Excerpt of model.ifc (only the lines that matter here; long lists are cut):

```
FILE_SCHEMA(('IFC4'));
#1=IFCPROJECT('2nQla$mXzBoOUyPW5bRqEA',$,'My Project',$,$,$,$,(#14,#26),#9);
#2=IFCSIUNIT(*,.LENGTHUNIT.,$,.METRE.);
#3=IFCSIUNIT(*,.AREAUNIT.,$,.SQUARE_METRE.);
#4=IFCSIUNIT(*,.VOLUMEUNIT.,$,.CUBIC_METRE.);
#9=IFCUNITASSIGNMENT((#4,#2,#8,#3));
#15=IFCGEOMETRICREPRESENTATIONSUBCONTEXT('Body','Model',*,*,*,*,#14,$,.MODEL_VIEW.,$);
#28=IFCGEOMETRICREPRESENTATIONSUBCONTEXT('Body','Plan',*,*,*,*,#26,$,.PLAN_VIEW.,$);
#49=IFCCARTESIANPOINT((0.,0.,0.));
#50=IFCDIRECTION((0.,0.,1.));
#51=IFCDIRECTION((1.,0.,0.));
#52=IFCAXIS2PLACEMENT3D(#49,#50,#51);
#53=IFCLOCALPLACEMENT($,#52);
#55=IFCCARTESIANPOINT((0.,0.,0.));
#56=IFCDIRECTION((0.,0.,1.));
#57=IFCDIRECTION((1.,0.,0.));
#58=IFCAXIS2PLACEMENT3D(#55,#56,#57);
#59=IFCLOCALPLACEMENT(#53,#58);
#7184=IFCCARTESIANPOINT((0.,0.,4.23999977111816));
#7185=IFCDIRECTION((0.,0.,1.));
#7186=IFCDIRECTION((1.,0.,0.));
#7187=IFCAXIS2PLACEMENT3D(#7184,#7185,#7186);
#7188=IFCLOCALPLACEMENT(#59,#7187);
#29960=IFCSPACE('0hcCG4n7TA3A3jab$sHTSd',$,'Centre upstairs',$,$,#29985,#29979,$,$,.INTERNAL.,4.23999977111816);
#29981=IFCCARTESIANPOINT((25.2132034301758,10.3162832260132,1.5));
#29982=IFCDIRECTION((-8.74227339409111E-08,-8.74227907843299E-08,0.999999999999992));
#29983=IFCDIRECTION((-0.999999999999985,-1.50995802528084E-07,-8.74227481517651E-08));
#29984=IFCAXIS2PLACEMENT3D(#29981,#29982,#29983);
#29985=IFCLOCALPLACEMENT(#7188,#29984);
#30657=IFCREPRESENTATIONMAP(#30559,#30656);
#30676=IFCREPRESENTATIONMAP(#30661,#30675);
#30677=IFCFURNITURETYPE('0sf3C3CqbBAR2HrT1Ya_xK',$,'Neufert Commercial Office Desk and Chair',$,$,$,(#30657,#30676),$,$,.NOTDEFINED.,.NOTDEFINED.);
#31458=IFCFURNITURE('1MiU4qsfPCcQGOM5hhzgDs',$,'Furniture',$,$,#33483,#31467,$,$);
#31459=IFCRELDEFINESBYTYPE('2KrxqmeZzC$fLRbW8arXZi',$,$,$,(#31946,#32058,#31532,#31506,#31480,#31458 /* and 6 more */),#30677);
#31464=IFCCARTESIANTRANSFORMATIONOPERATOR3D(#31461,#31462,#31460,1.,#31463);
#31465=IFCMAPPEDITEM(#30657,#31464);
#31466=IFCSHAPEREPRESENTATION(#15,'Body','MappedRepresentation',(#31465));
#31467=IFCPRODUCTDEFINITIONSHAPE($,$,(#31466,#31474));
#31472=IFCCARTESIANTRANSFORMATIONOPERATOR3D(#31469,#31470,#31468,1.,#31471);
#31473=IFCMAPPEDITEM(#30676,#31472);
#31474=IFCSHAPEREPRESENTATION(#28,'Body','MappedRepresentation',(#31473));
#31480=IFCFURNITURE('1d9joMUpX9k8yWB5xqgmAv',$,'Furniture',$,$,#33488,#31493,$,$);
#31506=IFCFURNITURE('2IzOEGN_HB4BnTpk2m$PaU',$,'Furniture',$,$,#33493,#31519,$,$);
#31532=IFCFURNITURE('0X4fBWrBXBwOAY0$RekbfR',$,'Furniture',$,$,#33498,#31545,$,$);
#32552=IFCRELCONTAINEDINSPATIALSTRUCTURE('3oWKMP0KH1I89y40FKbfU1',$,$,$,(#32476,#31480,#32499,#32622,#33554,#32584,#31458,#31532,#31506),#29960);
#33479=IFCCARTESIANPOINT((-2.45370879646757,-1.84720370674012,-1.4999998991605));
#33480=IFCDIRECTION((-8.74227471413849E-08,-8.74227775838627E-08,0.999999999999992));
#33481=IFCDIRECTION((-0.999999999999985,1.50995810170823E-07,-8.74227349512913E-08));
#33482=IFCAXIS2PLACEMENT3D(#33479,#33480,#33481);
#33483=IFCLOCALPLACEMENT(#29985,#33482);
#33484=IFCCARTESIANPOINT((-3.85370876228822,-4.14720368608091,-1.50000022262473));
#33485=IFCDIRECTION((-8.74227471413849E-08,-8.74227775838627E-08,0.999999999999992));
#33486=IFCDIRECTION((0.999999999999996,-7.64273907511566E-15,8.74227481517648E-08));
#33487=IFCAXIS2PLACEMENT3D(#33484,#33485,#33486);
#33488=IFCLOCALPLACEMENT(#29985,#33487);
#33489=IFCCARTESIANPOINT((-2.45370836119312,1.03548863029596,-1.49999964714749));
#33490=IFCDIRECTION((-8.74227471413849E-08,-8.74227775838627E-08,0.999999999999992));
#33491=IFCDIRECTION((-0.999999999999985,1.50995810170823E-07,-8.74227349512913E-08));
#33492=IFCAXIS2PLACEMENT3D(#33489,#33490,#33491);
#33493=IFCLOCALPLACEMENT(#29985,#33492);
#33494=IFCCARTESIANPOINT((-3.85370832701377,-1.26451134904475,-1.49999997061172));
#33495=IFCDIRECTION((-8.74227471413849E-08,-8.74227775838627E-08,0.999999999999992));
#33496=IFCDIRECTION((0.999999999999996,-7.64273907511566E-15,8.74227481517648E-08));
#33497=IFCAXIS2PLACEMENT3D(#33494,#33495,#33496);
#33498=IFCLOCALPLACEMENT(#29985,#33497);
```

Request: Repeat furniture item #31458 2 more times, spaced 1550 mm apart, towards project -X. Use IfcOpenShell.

```python
import numpy as np
import ifcopenshell
import ifcopenshell.api.geometry
import ifcopenshell.api.root
import ifcopenshell.util.element
import ifcopenshell.util.placement
import ifcopenshell.util.unit

model = ifcopenshell.open("model.ifc")
unit_scale = ifcopenshell.util.unit.calculate_unit_scale(model)

source = model.by_guid("1MiU4qsfPCcQGOM5hhzgDs")
base = ifcopenshell.util.placement.get_local_placement(source.ObjectPlacement)
step = np.array([-1.0, 0.0, 0.0]) * 1.55 / unit_scale

for i in range(1, 3):
    copy = ifcopenshell.api.root.copy_class(model, product=source)
    copy.Representation = ifcopenshell.util.element.copy_deep(
        model, source.Representation, exclude=["IfcGeometricRepresentationContext", "IfcRepresentationMap"]
    )
    matrix = base.copy()
    matrix[:3, 3] += i * step
    print("added at", matrix[:3, 3].round(3) + 0.0)
    ifcopenshell.api.geometry.edit_object_placement(model, product=copy, matrix=matrix, is_si=False)

model.write("model_rev.ifc")
```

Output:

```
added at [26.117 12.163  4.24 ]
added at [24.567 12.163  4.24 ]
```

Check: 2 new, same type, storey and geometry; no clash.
